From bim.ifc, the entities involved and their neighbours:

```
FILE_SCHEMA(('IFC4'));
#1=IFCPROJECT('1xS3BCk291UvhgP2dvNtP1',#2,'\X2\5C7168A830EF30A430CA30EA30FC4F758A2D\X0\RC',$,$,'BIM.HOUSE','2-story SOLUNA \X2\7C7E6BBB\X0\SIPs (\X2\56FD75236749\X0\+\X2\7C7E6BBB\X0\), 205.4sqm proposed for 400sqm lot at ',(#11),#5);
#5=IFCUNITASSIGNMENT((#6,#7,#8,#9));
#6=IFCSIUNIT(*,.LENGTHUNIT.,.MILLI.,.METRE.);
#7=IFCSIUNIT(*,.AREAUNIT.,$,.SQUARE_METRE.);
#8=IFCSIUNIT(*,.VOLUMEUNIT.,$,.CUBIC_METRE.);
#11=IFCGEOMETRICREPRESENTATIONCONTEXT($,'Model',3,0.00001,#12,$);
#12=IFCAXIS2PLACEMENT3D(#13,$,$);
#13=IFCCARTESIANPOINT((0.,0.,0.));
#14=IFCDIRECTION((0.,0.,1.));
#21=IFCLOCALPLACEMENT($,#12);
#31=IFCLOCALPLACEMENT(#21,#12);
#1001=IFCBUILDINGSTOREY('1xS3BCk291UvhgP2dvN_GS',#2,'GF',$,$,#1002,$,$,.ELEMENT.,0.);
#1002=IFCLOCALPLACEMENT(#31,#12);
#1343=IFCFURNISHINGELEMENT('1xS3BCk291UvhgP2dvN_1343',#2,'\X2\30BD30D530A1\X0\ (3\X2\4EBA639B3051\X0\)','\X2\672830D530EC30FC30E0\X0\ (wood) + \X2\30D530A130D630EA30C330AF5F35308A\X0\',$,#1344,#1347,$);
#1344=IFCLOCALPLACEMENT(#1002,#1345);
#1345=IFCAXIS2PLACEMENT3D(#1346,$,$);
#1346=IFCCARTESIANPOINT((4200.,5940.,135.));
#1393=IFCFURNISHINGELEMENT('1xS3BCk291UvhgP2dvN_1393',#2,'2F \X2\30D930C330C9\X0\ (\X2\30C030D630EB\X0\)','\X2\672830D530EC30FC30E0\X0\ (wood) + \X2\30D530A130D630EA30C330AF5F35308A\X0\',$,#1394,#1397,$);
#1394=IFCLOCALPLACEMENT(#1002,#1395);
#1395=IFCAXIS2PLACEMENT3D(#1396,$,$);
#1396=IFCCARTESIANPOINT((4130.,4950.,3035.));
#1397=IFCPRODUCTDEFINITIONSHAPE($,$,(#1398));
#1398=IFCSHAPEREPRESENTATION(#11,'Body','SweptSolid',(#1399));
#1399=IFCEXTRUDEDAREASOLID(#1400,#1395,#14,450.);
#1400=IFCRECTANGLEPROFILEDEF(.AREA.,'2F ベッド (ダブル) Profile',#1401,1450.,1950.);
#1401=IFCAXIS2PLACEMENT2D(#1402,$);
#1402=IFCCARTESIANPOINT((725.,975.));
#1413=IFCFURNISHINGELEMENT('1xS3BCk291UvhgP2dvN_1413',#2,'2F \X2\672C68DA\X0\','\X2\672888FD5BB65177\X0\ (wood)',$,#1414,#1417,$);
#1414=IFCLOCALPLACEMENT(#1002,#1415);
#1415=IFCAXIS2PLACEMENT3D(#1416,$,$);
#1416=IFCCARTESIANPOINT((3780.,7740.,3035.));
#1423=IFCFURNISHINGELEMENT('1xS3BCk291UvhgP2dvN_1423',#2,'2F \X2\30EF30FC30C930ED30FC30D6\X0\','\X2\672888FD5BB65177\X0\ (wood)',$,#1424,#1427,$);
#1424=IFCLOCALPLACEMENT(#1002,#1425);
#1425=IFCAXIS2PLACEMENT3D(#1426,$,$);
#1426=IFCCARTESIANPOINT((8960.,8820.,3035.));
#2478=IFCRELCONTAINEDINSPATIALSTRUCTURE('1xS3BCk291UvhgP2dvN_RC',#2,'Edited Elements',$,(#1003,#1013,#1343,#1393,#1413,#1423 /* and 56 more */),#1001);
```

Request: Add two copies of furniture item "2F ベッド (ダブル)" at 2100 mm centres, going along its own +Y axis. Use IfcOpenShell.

```python
import ifcopenshell
import ifcopenshell.api.geometry
import ifcopenshell.api.root
import ifcopenshell.util.element
import ifcopenshell.util.placement
import ifcopenshell.util.unit

model = ifcopenshell.open("bim.ifc")
unit_scale = ifcopenshell.util.unit.calculate_unit_scale(model)


def reuse_history(source, copy):
    """copy_class also copies each property set's owner history, people and application; keep the originals."""
    for rel in copy.IsDefinedBy:
        if rel.is_a("IfcRelDefinesByProperties") and (history := rel.RelatingPropertyDefinition.OwnerHistory):
            rel.RelatingPropertyDefinition.OwnerHistory = source.OwnerHistory
            ifcopenshell.util.element.remove_deep2(model, history)


source = model.by_guid("1xS3BCk291UvhgP2dvN_1393")
base = ifcopenshell.util.placement.get_local_placement(source.ObjectPlacement)
step = base[:3, 1] * 2.1 / unit_scale

for i in range(1, 3):
    copy = ifcopenshell.api.root.copy_class(model, product=source)
    copy.Representation = ifcopenshell.util.element.copy_deep(
        model, source.Representation, exclude=["IfcGeometricRepresentationContext", "IfcRepresentationMap"]
    )
    reuse_history(source, copy)
    matrix = base.copy()
    matrix[:3, 3] += i * step
    print("added at", matrix[:3, 3].round(3) + 0.0)
    ifcopenshell.api.geometry.edit_object_placement(model, product=copy, matrix=matrix, is_si=False)

model.write("bim_updated.ifc")
```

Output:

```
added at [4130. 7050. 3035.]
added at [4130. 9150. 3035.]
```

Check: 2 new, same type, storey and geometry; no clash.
